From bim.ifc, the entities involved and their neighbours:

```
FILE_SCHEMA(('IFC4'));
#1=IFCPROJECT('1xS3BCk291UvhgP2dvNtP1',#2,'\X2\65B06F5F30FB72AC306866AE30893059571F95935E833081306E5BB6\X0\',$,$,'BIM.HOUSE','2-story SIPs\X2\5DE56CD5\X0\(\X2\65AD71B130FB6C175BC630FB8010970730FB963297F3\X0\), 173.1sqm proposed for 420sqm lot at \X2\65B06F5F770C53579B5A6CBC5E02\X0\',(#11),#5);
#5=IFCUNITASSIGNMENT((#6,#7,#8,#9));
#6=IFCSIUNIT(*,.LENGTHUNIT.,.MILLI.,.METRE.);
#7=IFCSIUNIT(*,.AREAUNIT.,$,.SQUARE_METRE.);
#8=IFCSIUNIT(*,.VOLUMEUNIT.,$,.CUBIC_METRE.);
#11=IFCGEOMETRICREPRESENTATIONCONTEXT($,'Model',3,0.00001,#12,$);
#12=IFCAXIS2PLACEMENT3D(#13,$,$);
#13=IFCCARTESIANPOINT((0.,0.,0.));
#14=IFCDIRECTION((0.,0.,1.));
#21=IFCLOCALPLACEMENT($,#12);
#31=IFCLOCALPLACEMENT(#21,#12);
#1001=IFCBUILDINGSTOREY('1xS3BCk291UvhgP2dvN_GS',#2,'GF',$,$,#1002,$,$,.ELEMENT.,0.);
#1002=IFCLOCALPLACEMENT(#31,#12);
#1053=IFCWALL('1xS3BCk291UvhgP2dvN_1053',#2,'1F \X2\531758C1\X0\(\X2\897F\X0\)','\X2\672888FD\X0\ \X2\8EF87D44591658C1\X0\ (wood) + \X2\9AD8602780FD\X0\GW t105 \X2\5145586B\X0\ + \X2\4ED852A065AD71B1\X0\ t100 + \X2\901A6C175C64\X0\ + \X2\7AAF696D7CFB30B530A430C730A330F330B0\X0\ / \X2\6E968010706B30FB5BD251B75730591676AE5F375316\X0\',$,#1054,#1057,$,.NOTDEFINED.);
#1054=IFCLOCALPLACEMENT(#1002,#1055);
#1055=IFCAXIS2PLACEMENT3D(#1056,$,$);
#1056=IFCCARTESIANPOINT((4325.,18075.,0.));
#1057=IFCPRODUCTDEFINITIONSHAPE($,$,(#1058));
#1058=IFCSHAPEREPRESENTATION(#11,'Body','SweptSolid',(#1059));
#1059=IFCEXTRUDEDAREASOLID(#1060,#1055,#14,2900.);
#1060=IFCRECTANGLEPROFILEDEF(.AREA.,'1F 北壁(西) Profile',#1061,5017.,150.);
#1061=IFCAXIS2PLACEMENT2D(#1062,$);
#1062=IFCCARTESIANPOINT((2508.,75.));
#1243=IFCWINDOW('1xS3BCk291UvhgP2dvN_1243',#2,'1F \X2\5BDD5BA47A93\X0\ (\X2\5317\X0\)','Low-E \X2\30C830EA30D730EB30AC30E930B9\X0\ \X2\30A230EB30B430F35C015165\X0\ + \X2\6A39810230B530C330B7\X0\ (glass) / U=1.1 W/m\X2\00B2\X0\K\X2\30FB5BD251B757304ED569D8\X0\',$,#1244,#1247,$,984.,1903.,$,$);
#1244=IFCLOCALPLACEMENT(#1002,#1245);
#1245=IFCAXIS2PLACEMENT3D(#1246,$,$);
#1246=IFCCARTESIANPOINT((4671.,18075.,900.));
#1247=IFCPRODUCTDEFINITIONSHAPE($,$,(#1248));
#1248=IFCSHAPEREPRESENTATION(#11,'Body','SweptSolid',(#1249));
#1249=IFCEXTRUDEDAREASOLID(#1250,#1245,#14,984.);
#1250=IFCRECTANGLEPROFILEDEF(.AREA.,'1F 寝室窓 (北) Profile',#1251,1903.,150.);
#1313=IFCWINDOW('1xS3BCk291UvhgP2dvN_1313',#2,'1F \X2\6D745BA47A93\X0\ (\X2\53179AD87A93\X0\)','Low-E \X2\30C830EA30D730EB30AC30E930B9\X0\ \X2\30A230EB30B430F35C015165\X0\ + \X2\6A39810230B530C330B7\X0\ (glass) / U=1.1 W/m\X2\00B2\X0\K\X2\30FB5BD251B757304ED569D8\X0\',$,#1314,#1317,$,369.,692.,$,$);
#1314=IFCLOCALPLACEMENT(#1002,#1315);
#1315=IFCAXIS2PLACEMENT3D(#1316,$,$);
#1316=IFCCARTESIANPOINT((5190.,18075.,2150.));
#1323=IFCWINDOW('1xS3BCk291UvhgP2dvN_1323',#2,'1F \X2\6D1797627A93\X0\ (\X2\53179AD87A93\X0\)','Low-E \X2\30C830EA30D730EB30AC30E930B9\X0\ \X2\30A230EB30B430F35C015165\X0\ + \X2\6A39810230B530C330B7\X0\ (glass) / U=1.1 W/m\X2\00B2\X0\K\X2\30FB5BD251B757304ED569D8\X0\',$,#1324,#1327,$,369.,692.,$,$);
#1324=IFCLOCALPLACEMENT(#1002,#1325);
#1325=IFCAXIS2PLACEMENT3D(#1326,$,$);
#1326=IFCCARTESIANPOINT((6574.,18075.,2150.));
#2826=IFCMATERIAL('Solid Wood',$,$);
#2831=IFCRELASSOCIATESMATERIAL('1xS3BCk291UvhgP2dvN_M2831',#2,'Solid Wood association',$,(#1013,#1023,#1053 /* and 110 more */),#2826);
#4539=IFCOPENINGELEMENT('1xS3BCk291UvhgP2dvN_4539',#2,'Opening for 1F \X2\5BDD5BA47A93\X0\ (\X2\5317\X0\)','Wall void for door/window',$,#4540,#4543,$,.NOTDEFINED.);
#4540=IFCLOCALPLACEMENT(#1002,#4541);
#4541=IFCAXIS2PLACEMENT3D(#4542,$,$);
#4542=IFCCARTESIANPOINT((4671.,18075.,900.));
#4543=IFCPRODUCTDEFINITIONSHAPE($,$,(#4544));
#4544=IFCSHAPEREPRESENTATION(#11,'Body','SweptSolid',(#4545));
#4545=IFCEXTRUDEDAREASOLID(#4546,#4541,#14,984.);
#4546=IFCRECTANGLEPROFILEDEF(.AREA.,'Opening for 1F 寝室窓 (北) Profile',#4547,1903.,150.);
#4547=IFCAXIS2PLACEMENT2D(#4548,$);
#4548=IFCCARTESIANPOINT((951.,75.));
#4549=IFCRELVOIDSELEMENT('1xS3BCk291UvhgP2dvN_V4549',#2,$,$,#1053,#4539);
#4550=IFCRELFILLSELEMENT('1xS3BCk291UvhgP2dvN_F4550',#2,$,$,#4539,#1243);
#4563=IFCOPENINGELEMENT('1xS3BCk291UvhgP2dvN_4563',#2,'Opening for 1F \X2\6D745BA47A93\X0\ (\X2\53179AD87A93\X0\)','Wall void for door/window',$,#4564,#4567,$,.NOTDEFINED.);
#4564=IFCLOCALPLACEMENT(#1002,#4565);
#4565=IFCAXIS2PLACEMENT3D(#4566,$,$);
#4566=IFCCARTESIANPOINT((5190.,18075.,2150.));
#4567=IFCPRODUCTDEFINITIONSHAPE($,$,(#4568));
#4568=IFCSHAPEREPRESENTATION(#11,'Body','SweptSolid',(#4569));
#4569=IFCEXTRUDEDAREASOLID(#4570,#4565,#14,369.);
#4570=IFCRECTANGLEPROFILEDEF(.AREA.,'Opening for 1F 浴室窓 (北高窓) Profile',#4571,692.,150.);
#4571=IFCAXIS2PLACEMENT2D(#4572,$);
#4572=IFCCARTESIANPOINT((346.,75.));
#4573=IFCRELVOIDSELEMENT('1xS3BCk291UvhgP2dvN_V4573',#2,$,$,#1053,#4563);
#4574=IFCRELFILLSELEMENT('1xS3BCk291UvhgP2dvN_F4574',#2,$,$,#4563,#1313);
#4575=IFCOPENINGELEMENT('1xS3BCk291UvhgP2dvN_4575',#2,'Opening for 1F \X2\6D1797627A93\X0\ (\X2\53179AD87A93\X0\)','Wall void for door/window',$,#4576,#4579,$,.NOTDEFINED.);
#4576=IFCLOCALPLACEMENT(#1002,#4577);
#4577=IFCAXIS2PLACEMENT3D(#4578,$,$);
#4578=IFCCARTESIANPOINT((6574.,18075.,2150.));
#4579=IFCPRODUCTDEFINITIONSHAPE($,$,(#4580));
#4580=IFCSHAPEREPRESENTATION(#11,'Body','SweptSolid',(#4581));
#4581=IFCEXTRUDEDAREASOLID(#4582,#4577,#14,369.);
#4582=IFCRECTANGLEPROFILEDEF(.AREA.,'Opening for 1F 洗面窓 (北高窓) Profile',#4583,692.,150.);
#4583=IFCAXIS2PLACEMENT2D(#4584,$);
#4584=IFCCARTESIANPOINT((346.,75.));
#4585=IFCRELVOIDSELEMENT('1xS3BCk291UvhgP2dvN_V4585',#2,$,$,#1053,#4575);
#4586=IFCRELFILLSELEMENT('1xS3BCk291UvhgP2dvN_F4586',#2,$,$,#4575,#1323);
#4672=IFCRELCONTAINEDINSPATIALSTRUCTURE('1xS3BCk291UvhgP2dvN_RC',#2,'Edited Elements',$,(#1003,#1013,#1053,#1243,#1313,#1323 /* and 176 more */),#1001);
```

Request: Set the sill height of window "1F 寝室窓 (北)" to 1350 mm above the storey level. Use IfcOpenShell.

```python
import numpy as np
import ifcopenshell
import ifcopenshell.api.geometry
import ifcopenshell.geom
import ifcopenshell.util.element
import ifcopenshell.util.placement
import ifcopenshell.util.shape
import ifcopenshell.util.unit

model = ifcopenshell.open("bim.ifc")
unit_scale = ifcopenshell.util.unit.calculate_unit_scale(model)

window = model.by_id(1243)
opening = window.FillsVoids[0].RelatingOpeningElement
storey = ifcopenshell.util.element.get_container(window, ifc_class="IfcBuildingStorey")
level = ifcopenshell.util.placement.get_local_placement(storey.ObjectPlacement)[2, 3]

# The opening's origin need not be at the sill, so measure its lowest point.
shape = ifcopenshell.geom.create_shape(ifcopenshell.geom.settings(), opening)
bottom = ifcopenshell.util.shape.get_shape_bottom_elevation(shape, shape.geometry) / unit_scale
dz = level + 1.35 / unit_scale - bottom

shift = np.array([0.0, 0.0, dz])
# The window is not placed relative to its opening, so move both.
for product in (opening, window):
    matrix = ifcopenshell.util.placement.get_local_placement(product.ObjectPlacement)
    matrix[:3, 3] += shift
    ifcopenshell.api.geometry.edit_object_placement(model, product=product, matrix=matrix, is_si=False)

print(f"moved by {dz * unit_scale:+.3f} m")

model.write("bim_updated.ifc")
```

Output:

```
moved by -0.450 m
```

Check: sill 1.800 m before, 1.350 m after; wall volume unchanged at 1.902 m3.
